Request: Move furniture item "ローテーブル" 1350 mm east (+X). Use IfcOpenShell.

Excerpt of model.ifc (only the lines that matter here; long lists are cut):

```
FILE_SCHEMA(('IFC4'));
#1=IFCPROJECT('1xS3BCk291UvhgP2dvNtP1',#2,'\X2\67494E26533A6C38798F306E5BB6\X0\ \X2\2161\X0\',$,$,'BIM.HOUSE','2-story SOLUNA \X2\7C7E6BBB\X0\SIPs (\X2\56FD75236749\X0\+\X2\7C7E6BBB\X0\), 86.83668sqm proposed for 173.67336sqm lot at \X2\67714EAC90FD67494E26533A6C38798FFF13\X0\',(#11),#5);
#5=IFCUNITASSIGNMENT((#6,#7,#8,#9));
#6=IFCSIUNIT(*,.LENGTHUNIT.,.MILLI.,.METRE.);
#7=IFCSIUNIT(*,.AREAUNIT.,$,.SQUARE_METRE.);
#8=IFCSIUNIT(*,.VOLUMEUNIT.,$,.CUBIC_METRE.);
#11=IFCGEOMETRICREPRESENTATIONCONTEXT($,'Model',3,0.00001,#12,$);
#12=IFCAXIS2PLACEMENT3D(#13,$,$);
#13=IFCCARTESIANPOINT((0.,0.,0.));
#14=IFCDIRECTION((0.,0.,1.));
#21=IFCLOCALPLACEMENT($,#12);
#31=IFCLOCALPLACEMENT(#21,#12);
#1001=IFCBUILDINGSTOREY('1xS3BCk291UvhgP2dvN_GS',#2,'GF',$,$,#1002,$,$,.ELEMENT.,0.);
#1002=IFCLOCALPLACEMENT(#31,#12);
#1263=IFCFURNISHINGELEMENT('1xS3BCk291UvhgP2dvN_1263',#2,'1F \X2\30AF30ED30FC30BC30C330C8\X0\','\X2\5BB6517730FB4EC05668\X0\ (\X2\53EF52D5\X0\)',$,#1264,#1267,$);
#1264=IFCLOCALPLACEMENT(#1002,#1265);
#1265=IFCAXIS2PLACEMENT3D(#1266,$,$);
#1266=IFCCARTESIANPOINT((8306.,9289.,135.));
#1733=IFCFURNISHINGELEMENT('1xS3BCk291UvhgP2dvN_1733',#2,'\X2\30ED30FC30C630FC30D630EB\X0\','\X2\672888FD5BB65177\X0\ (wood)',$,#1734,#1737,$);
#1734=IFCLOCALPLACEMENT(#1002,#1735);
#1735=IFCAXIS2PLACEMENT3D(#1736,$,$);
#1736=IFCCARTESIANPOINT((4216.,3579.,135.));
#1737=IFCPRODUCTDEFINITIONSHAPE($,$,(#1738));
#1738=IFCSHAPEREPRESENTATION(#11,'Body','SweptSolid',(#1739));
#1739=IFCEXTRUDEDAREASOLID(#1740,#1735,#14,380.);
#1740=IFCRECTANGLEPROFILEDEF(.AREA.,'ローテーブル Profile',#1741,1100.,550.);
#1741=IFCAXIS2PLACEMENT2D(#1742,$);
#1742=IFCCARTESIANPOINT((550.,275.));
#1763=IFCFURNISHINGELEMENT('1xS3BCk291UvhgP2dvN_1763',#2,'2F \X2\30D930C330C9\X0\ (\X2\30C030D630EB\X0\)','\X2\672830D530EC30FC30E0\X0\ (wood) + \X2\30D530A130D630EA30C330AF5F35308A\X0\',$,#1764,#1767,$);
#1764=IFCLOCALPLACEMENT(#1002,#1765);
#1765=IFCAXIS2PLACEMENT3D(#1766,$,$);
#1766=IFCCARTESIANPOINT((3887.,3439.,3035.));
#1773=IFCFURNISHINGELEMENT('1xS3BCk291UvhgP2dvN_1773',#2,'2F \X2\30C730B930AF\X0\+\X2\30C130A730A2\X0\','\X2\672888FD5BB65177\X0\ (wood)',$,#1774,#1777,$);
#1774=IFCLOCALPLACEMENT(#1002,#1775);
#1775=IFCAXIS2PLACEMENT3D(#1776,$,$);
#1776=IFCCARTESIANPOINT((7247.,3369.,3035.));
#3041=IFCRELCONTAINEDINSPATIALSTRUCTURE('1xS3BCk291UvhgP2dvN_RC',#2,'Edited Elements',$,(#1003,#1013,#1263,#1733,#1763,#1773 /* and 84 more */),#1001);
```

```python
import ifcopenshell
import ifcopenshell.api.geometry
import ifcopenshell.util.placement
import ifcopenshell.util.unit

model = ifcopenshell.open("model.ifc")
unit_scale = ifcopenshell.util.unit.calculate_unit_scale(model)

item = model.by_guid("1xS3BCk291UvhgP2dvN_1733")
matrix = ifcopenshell.util.placement.get_local_placement(item.ObjectPlacement)
matrix[0, 3] += 1.35 / unit_scale
ifcopenshell.api.geometry.edit_object_placement(model, product=item, matrix=matrix, is_si=False)

print(ifcopenshell.util.placement.get_local_placement(item.ObjectPlacement).round(3) + 0.0)

model.write("model_rev.ifc")
```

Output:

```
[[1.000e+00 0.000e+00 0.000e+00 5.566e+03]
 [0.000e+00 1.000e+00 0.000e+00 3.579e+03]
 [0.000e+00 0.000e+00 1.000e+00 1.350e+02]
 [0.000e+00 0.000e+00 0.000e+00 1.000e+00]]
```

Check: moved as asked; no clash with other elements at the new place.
